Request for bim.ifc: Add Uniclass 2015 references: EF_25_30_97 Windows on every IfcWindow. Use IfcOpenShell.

First a look at what the model holds.

```python
import ifcopenshell

model = ifcopenshell.open("bim.ifc")
print(model.schema)
print("classifications:", [c.Name for c in model.by_type("IfcClassification")])
for ifc_class in ("IfcDoor", "IfcRoof", "IfcStair", "IfcWall", "IfcWindow"):
    print(ifc_class, len(model.by_type(ifc_class)))
```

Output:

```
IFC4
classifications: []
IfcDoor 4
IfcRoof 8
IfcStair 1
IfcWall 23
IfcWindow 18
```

```python
import ifcopenshell
import ifcopenshell.api.classification

model = ifcopenshell.open("bim.ifc")

system = ifcopenshell.api.classification.add_classification(model, classification="Uniclass 2015")

codes = {
    "IfcWindow": ("EF_25_30_97", "Windows"),
}
for ifc_class, (code, name) in codes.items():
    products = model.by_type(ifc_class)
    ifcopenshell.api.classification.add_reference(
        model, products=products, classification=system, identification=code, name=name
    )
    print(code, len(products))

model.write("bim_edited.ifc")
```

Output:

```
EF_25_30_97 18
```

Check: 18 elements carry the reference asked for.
